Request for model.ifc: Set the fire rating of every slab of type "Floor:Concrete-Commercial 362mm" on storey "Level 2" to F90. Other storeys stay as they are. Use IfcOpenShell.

First a look at what the model holds.

```python
import ifcopenshell
import ifcopenshell.util.element

model = ifcopenshell.open("model.ifc")
print(model.schema)
storey = next(s for s in model.by_type("IfcBuildingStorey") if s.Name == "Level 2")
slabs = [e for e in ifcopenshell.util.element.get_decomposition(storey) if e.is_a("IfcSlab")]
seen = {}
for e in slabs:
    element_type = ifcopenshell.util.element.get_type(e)
    key = (element_type.Name if element_type != e and element_type else None, ifcopenshell.util.element.get_pset(e, "Pset_SlabCommon", "FireRating"))
    seen[key] = seen.get(key, 0) + 1
for (name, value), count in sorted(seen.items(), key=str):
    print(count, "x", name, "|", value)
```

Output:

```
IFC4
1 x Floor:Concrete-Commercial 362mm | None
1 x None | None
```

```python
import ifcopenshell
import ifcopenshell.api.pset
import ifcopenshell.util.element

model = ifcopenshell.open("model.ifc")

storey = next(s for s in model.by_type("IfcBuildingStorey") if s.Name == "Level 2")
slabs = [e for e in ifcopenshell.util.element.get_decomposition(storey) if e.is_a("IfcSlab")]

count = 0
for e in slabs:
    element_type = ifcopenshell.util.element.get_type(e)
    if element_type in (None, e) or element_type.Name != "Floor:Concrete-Commercial 362mm":
        continue
    # add_pset returns the element's existing set when there is one.
    pset = ifcopenshell.api.pset.add_pset(model, product=e, name="Pset_SlabCommon")
    ifcopenshell.api.pset.edit_pset(model, pset=pset, properties={"FireRating": "F90"})
    count += 1

print(count, "slabs updated")

model.write("model_updated.ifc")
```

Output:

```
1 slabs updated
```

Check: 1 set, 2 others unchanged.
